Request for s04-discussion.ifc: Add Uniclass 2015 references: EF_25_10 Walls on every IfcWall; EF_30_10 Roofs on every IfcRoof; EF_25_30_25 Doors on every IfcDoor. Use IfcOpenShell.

First a look at what the model holds.

```python
import ifcopenshell

model = ifcopenshell.open("s04-discussion.ifc")
print(model.schema)
print("classifications:", [c.Name for c in model.by_type("IfcClassification")])
for ifc_class in ("IfcDoor", "IfcRoof", "IfcStair", "IfcWall", "IfcWindow"):
    print(ifc_class, len(model.by_type(ifc_class)))
```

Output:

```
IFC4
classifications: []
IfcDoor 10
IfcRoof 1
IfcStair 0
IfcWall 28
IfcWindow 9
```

```python
import ifcopenshell
import ifcopenshell.api.classification

model = ifcopenshell.open("s04-discussion.ifc")

system = ifcopenshell.api.classification.add_classification(model, classification="Uniclass 2015")

codes = {
    "IfcWall": ("EF_25_10", "Walls"),
    "IfcRoof": ("EF_30_10", "Roofs"),
    "IfcDoor": ("EF_25_30_25", "Doors"),
}
for ifc_class, (code, name) in codes.items():
    products = model.by_type(ifc_class)
    ifcopenshell.api.classification.add_reference(
        model, products=products, classification=system, identification=code, name=name
    )
    print(code, len(products))

model.write("s04-discussion_rev.ifc")
```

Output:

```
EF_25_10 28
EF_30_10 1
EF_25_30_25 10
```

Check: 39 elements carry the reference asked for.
